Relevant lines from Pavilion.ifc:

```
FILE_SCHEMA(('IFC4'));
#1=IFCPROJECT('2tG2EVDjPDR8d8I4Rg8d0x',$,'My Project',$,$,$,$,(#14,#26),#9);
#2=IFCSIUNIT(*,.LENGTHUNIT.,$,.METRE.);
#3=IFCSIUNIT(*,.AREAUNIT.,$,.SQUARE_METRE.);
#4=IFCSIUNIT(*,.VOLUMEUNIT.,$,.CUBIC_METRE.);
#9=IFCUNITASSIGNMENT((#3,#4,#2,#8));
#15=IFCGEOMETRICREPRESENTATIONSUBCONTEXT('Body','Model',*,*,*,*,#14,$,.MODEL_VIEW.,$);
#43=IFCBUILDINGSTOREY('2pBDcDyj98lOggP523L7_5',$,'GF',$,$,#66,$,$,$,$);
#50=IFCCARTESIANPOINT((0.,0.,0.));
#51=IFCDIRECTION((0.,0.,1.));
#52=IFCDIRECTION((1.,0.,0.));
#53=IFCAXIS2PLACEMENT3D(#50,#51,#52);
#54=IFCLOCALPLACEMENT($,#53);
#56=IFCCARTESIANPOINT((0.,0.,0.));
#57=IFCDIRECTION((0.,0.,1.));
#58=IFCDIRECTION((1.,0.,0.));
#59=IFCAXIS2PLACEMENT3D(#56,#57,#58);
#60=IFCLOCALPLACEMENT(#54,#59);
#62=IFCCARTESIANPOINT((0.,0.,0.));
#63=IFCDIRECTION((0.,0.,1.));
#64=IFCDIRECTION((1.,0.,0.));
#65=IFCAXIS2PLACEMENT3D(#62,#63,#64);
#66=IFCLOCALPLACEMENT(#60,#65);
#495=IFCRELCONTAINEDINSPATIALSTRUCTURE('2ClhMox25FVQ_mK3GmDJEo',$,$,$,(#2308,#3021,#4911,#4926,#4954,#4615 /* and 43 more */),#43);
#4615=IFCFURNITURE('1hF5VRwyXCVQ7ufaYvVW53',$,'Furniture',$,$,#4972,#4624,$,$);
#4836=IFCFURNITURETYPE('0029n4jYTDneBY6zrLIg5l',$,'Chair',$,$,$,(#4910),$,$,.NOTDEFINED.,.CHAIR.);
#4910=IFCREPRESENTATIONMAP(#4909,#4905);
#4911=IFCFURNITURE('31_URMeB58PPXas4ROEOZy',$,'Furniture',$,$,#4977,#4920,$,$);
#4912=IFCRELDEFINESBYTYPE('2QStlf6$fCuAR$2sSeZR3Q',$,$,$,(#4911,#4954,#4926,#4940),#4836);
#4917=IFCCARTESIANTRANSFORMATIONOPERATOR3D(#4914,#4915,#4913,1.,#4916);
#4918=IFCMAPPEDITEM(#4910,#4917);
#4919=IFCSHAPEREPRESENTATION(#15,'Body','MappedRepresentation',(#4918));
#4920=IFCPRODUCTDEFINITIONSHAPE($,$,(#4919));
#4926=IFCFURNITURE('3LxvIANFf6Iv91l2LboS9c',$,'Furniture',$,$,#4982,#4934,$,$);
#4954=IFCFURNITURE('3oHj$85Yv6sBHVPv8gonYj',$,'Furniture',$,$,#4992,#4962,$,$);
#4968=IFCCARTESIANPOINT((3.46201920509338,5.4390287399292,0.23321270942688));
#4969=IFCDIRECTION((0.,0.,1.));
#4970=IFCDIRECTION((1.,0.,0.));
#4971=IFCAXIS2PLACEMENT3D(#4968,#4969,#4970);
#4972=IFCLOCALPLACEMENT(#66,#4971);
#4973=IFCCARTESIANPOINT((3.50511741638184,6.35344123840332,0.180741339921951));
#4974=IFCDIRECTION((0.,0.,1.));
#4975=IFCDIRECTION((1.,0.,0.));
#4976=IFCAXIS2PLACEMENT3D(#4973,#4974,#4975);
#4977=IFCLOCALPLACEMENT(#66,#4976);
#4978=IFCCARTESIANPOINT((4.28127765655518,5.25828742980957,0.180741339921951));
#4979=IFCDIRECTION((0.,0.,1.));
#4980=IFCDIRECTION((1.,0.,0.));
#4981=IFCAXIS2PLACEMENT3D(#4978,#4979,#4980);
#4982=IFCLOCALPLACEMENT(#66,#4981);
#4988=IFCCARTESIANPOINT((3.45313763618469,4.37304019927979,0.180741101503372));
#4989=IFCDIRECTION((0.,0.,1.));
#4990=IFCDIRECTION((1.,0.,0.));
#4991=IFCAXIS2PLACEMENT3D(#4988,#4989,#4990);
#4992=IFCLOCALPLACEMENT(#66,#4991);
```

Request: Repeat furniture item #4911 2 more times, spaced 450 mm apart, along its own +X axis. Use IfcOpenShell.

```python
import ifcopenshell
import ifcopenshell.api.geometry
import ifcopenshell.api.root
import ifcopenshell.util.element
import ifcopenshell.util.placement
import ifcopenshell.util.unit

model = ifcopenshell.open("Pavilion.ifc")
unit_scale = ifcopenshell.util.unit.calculate_unit_scale(model)

source = model.by_id(4911)
base = ifcopenshell.util.placement.get_local_placement(source.ObjectPlacement)
step = base[:3, 0] * 0.45 / unit_scale

for i in range(1, 3):
    copy = ifcopenshell.api.root.copy_class(model, product=source)
    copy.Representation = ifcopenshell.util.element.copy_deep(
        model, source.Representation, exclude=["IfcGeometricRepresentationContext", "IfcRepresentationMap"]
    )
    matrix = base.copy()
    matrix[:3, 3] += i * step
    print("added at", matrix[:3, 3].round(3) + 0.0)
    ifcopenshell.api.geometry.edit_object_placement(model, product=copy, matrix=matrix, is_si=False)

model.write("Pavilion-out.ifc")
```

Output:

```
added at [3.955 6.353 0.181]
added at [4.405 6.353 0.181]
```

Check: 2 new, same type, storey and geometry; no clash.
